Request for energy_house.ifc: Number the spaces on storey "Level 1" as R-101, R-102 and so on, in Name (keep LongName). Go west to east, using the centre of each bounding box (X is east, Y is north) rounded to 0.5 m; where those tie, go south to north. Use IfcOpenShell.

First a look at what the model holds.

```python
import ifcopenshell
import ifcopenshell.util.element
import ifcopenshell.util.placement

model = ifcopenshell.open("energy_house.ifc")
print(model.schema)
storey = next(s for s in model.by_type("IfcBuildingStorey") if s.Name == "Level 1")
spaces = [e for e in ifcopenshell.util.element.get_decomposition(storey) if e.is_a("IfcSpace")]
for e in sorted(spaces, key=lambda e: e.id()):
    origin = ifcopenshell.util.placement.get_local_placement(e.ObjectPlacement)[:3, 3]
    print(e.id(), e.Name, e.LongName, origin.round(2) + 0.0, sep=" | ")
```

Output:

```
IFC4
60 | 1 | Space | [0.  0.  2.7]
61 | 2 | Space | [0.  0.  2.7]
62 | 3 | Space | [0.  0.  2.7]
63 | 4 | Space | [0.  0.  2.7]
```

```python
import ifcopenshell
import ifcopenshell.geom
import ifcopenshell.util.element
import ifcopenshell.util.shape

model = ifcopenshell.open("energy_house.ifc")
settings = ifcopenshell.geom.settings()
settings.set("use-world-coords", True)


def centre(element):
    shape = ifcopenshell.geom.create_shape(settings, element)
    return ifcopenshell.util.shape.get_bbox_centroid(shape.geometry)


storey = next(s for s in model.by_type("IfcBuildingStorey") if s.Name == "Level 1")
spaces = [e for e in ifcopenshell.util.element.get_decomposition(storey) if e.is_a("IfcSpace")]

# Insertion points can sit at a corner or the storey origin, so sort by the geometry (in metres).
centres = {e: centre(e) for e in spaces}
spaces.sort(key=lambda e: (round(centres[e][0] / 0.5), centres[e][1]))

for i, e in enumerate(spaces, start=1):
    number = f"R-1{i:02d}"
    e.Name = number
    print(e.id(), number)

model.write("energy_house_edited.ifc")
```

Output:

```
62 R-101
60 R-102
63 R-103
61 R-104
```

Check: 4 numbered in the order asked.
